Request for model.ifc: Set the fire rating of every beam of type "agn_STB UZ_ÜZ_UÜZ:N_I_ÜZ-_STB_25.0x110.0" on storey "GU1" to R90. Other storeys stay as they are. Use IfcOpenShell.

First a look at what the model holds.

```python
import ifcopenshell
import ifcopenshell.util.element

model = ifcopenshell.open("model.ifc")
print(model.schema)
storey = next(s for s in model.by_type("IfcBuildingStorey") if s.Name == "GU1")
beams = [e for e in ifcopenshell.util.element.get_decomposition(storey) if e.is_a("IfcBeam")]
seen = {}
for e in beams:
    element_type = ifcopenshell.util.element.get_type(e)
    key = (element_type.Name if element_type != e and element_type else None, ifcopenshell.util.element.get_pset(e, "Pset_BeamCommon", "FireRating"))
    seen[key] = seen.get(key, 0) + 1
for (name, value), count in sorted(seen.items(), key=str):
    print(count, "x", name, "|", value)
```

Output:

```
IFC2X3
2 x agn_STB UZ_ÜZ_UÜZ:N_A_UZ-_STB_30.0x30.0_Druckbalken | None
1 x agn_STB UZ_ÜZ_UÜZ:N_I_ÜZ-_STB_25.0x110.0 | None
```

```python
import ifcopenshell
import ifcopenshell.api.pset
import ifcopenshell.util.element

model = ifcopenshell.open("model.ifc")

storey = next(s for s in model.by_type("IfcBuildingStorey") if s.Name == "GU1")
beams = [e for e in ifcopenshell.util.element.get_decomposition(storey) if e.is_a("IfcBeam")]

count = 0
for e in beams:
    element_type = ifcopenshell.util.element.get_type(e)
    if element_type in (None, e) or element_type.Name != "agn_STB UZ_ÜZ_UÜZ:N_I_ÜZ-_STB_25.0x110.0":
        continue
    found = ifcopenshell.util.element.get_pset(e, "Pset_BeamCommon", should_inherit=False)
    if found:
        pset = model.by_id(found["id"])
        if len(ifcopenshell.util.element.get_elements_by_pset(pset)) > 1:
            pset = ifcopenshell.api.pset.unshare_pset(model, products=[e], pset=pset)[0]
    else:
        pset = ifcopenshell.api.pset.add_pset(model, product=e, name="Pset_BeamCommon")
    ifcopenshell.api.pset.edit_pset(model, pset=pset, properties={"FireRating": "R90"})
    count += 1

print(count, "beams updated")

model.write("model-out.ifc")
```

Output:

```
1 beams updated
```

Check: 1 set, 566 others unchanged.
